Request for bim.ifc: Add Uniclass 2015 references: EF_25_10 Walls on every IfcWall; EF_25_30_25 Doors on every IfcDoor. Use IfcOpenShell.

First a look at what the model holds.

```python
import ifcopenshell

model = ifcopenshell.open("bim.ifc")
print(model.schema)
print("classifications:", [c.Name for c in model.by_type("IfcClassification")])
for ifc_class in ("IfcDoor", "IfcRoof", "IfcStair", "IfcWall", "IfcWindow"):
    print(ifc_class, len(model.by_type(ifc_class)))
```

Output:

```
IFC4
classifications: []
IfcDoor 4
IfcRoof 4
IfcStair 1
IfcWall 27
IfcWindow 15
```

```python
import ifcopenshell
import ifcopenshell.api.classification

model = ifcopenshell.open("bim.ifc")

system = ifcopenshell.api.classification.add_classification(model, classification="Uniclass 2015")

codes = {
    "IfcWall": ("EF_25_10", "Walls"),
    "IfcDoor": ("EF_25_30_25", "Doors"),
}
for ifc_class, (code, name) in codes.items():
    products = model.by_type(ifc_class)
    ifcopenshell.api.classification.add_reference(
        model, products=products, classification=system, identification=code, name=name
    )
    print(code, len(products))

model.write("bim_v2.ifc")
```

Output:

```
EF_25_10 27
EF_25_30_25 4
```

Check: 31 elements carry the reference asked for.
